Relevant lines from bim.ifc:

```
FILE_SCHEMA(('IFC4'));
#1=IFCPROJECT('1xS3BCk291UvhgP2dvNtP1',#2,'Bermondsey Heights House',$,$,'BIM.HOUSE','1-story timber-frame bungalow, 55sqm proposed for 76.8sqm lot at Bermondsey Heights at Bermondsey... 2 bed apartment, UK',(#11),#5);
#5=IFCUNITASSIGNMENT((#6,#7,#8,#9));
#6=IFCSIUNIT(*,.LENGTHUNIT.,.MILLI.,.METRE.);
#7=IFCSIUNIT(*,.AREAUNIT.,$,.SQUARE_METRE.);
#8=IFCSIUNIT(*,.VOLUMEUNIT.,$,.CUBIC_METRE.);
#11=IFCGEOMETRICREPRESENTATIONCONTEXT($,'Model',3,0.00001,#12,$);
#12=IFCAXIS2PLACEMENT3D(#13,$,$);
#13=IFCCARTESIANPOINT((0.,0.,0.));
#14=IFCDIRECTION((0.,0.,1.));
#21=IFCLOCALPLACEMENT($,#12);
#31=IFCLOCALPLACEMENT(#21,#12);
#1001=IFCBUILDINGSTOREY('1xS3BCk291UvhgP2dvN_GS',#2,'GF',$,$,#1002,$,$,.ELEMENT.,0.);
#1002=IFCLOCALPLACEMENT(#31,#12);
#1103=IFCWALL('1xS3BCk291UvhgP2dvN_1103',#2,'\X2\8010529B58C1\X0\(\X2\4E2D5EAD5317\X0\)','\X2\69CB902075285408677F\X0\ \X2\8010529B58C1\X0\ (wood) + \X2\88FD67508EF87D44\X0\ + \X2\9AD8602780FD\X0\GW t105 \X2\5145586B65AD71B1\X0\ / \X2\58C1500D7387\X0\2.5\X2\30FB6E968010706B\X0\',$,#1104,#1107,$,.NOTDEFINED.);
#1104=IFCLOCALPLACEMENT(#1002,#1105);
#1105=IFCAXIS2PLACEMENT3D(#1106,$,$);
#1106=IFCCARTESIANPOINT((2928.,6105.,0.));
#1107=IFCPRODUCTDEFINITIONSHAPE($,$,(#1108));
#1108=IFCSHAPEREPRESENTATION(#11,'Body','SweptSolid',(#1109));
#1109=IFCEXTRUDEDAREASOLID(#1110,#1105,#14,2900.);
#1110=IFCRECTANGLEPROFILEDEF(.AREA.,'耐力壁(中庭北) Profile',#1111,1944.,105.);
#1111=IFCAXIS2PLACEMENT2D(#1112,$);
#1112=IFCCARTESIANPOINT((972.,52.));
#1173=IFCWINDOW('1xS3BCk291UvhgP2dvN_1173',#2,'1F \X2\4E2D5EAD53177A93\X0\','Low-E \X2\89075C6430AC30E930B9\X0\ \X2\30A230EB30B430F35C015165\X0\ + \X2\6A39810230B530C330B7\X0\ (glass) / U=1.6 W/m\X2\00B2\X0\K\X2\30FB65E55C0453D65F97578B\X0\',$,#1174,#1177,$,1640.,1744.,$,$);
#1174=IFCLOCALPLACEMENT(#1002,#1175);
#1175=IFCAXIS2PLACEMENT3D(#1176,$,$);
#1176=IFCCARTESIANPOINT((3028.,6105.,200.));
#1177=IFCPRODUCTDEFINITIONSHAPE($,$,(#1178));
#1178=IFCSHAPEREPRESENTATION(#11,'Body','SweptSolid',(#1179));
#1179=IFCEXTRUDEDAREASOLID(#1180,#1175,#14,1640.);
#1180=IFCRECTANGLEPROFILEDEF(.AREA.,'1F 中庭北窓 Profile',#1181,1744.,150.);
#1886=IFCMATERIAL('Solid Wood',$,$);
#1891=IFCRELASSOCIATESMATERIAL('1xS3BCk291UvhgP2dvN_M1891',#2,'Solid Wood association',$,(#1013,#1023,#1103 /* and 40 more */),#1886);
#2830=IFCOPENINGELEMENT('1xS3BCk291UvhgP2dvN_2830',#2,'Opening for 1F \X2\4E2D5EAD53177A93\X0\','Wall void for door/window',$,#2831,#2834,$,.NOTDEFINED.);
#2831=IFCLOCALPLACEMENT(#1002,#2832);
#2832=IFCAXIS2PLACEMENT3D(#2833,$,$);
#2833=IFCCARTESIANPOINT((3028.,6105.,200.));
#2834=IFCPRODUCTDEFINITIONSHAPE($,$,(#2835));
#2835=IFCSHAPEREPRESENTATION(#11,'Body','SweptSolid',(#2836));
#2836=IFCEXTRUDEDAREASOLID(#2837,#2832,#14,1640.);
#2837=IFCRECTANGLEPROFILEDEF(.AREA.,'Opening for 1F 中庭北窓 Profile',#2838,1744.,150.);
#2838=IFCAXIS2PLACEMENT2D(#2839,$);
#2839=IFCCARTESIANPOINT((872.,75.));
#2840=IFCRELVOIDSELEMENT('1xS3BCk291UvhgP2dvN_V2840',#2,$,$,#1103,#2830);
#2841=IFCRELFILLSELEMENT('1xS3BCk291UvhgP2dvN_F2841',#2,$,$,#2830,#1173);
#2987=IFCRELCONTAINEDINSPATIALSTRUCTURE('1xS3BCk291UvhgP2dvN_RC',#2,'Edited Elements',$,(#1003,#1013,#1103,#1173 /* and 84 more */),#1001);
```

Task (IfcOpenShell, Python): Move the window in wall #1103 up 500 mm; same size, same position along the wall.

```python
import numpy as np
import ifcopenshell
import ifcopenshell.api.geometry
import ifcopenshell.util.placement
import ifcopenshell.util.unit

model = ifcopenshell.open("bim.ifc")
unit_scale = ifcopenshell.util.unit.calculate_unit_scale(model)

window = model.by_id(1173)
opening = window.FillsVoids[0].RelatingOpeningElement
dz = 500.0

shift = np.array([0.0, 0.0, dz])
# The window is not placed relative to its opening, so move both.
for product in (opening, window):
    matrix = ifcopenshell.util.placement.get_local_placement(product.ObjectPlacement)
    matrix[:3, 3] += shift
    ifcopenshell.api.geometry.edit_object_placement(model, product=product, matrix=matrix, is_si=False)

print(f"moved by {dz * unit_scale:+.3f} m")

model.write("bim_updated.ifc")
```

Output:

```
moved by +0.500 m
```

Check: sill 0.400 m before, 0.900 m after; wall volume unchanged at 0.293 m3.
